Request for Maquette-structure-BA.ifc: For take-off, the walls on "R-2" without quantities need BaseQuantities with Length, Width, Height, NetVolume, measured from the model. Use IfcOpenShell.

First a look at what the model holds.

```python
import ifcopenshell
import ifcopenshell.util.element
import ifcopenshell.util.unit

model = ifcopenshell.open("Maquette-structure-BA.ifc")
print(model.schema)
for unit_type in ("LENGTHUNIT", "AREAUNIT", "VOLUMEUNIT"):
    print(unit_type, ifcopenshell.util.unit.calculate_unit_scale(model, unit_type))
storey = next(s for s in model.by_type("IfcBuildingStorey") if s.Name == "R-2")
walls = [e for e in ifcopenshell.util.element.get_decomposition(storey) if e.is_a("IfcWall")]
for e in sorted(walls, key=lambda e: e.id()):
    print(e.id(), e.is_a(), e.Name, list(ifcopenshell.util.element.get_psets(e, qtos_only=True)), sep=" | ")
```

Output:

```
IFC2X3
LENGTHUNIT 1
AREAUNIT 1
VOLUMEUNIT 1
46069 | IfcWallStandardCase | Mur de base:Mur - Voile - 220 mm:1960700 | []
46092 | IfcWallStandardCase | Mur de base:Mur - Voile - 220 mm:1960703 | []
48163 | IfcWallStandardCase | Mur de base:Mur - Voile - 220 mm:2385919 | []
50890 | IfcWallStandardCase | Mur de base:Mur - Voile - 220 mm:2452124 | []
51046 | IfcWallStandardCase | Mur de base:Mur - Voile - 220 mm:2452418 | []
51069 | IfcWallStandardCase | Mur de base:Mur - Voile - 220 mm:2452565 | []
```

```python
import ifcopenshell
import ifcopenshell.api.pset
import ifcopenshell.geom
import ifcopenshell.util.element
import ifcopenshell.util.shape
import ifcopenshell.util.unit

model = ifcopenshell.open("Maquette-structure-BA.ifc")
unit_scale = ifcopenshell.util.unit.calculate_unit_scale(model)
volume_scale = ifcopenshell.util.unit.calculate_unit_scale(model, "VOLUMEUNIT")
settings = ifcopenshell.geom.settings()

storey = next(s for s in model.by_type("IfcBuildingStorey") if s.Name == "R-2")
walls = [e for e in ifcopenshell.util.element.get_decomposition(storey) if e.is_a("IfcWall")]

for e in sorted(walls, key=lambda e: e.id()):
    if ifcopenshell.util.element.get_psets(e, qtos_only=True, should_inherit=False):
        continue
    # Geometry comes back in metres, in the element's own axes.
    shape = ifcopenshell.geom.create_shape(settings, e)
    values = {
        "Length": ifcopenshell.util.shape.get_x(shape.geometry) / unit_scale,
        "Width": ifcopenshell.util.shape.get_y(shape.geometry) / unit_scale,
        "Height": ifcopenshell.util.shape.get_z(shape.geometry) / unit_scale,
        "NetVolume": ifcopenshell.util.shape.get_volume(shape.geometry) / volume_scale,
    }
    qto = ifcopenshell.api.pset.add_qto(model, product=e, name="BaseQuantities")
    ifcopenshell.api.pset.edit_qto(model, qto=qto, properties=values)
    print(e.id(), {k: round(v, 3) for k, v in values.items()})

model.write("Maquette-structure-BA-out.ifc")
```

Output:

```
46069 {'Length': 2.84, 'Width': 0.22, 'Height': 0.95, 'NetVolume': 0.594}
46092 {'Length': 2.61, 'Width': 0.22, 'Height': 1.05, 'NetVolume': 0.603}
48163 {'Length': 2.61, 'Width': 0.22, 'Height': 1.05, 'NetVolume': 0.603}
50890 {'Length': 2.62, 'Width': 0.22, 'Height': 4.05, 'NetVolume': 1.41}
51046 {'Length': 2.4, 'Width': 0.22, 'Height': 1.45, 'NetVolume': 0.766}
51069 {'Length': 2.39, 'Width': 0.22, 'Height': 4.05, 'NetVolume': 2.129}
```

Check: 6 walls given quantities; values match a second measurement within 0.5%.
